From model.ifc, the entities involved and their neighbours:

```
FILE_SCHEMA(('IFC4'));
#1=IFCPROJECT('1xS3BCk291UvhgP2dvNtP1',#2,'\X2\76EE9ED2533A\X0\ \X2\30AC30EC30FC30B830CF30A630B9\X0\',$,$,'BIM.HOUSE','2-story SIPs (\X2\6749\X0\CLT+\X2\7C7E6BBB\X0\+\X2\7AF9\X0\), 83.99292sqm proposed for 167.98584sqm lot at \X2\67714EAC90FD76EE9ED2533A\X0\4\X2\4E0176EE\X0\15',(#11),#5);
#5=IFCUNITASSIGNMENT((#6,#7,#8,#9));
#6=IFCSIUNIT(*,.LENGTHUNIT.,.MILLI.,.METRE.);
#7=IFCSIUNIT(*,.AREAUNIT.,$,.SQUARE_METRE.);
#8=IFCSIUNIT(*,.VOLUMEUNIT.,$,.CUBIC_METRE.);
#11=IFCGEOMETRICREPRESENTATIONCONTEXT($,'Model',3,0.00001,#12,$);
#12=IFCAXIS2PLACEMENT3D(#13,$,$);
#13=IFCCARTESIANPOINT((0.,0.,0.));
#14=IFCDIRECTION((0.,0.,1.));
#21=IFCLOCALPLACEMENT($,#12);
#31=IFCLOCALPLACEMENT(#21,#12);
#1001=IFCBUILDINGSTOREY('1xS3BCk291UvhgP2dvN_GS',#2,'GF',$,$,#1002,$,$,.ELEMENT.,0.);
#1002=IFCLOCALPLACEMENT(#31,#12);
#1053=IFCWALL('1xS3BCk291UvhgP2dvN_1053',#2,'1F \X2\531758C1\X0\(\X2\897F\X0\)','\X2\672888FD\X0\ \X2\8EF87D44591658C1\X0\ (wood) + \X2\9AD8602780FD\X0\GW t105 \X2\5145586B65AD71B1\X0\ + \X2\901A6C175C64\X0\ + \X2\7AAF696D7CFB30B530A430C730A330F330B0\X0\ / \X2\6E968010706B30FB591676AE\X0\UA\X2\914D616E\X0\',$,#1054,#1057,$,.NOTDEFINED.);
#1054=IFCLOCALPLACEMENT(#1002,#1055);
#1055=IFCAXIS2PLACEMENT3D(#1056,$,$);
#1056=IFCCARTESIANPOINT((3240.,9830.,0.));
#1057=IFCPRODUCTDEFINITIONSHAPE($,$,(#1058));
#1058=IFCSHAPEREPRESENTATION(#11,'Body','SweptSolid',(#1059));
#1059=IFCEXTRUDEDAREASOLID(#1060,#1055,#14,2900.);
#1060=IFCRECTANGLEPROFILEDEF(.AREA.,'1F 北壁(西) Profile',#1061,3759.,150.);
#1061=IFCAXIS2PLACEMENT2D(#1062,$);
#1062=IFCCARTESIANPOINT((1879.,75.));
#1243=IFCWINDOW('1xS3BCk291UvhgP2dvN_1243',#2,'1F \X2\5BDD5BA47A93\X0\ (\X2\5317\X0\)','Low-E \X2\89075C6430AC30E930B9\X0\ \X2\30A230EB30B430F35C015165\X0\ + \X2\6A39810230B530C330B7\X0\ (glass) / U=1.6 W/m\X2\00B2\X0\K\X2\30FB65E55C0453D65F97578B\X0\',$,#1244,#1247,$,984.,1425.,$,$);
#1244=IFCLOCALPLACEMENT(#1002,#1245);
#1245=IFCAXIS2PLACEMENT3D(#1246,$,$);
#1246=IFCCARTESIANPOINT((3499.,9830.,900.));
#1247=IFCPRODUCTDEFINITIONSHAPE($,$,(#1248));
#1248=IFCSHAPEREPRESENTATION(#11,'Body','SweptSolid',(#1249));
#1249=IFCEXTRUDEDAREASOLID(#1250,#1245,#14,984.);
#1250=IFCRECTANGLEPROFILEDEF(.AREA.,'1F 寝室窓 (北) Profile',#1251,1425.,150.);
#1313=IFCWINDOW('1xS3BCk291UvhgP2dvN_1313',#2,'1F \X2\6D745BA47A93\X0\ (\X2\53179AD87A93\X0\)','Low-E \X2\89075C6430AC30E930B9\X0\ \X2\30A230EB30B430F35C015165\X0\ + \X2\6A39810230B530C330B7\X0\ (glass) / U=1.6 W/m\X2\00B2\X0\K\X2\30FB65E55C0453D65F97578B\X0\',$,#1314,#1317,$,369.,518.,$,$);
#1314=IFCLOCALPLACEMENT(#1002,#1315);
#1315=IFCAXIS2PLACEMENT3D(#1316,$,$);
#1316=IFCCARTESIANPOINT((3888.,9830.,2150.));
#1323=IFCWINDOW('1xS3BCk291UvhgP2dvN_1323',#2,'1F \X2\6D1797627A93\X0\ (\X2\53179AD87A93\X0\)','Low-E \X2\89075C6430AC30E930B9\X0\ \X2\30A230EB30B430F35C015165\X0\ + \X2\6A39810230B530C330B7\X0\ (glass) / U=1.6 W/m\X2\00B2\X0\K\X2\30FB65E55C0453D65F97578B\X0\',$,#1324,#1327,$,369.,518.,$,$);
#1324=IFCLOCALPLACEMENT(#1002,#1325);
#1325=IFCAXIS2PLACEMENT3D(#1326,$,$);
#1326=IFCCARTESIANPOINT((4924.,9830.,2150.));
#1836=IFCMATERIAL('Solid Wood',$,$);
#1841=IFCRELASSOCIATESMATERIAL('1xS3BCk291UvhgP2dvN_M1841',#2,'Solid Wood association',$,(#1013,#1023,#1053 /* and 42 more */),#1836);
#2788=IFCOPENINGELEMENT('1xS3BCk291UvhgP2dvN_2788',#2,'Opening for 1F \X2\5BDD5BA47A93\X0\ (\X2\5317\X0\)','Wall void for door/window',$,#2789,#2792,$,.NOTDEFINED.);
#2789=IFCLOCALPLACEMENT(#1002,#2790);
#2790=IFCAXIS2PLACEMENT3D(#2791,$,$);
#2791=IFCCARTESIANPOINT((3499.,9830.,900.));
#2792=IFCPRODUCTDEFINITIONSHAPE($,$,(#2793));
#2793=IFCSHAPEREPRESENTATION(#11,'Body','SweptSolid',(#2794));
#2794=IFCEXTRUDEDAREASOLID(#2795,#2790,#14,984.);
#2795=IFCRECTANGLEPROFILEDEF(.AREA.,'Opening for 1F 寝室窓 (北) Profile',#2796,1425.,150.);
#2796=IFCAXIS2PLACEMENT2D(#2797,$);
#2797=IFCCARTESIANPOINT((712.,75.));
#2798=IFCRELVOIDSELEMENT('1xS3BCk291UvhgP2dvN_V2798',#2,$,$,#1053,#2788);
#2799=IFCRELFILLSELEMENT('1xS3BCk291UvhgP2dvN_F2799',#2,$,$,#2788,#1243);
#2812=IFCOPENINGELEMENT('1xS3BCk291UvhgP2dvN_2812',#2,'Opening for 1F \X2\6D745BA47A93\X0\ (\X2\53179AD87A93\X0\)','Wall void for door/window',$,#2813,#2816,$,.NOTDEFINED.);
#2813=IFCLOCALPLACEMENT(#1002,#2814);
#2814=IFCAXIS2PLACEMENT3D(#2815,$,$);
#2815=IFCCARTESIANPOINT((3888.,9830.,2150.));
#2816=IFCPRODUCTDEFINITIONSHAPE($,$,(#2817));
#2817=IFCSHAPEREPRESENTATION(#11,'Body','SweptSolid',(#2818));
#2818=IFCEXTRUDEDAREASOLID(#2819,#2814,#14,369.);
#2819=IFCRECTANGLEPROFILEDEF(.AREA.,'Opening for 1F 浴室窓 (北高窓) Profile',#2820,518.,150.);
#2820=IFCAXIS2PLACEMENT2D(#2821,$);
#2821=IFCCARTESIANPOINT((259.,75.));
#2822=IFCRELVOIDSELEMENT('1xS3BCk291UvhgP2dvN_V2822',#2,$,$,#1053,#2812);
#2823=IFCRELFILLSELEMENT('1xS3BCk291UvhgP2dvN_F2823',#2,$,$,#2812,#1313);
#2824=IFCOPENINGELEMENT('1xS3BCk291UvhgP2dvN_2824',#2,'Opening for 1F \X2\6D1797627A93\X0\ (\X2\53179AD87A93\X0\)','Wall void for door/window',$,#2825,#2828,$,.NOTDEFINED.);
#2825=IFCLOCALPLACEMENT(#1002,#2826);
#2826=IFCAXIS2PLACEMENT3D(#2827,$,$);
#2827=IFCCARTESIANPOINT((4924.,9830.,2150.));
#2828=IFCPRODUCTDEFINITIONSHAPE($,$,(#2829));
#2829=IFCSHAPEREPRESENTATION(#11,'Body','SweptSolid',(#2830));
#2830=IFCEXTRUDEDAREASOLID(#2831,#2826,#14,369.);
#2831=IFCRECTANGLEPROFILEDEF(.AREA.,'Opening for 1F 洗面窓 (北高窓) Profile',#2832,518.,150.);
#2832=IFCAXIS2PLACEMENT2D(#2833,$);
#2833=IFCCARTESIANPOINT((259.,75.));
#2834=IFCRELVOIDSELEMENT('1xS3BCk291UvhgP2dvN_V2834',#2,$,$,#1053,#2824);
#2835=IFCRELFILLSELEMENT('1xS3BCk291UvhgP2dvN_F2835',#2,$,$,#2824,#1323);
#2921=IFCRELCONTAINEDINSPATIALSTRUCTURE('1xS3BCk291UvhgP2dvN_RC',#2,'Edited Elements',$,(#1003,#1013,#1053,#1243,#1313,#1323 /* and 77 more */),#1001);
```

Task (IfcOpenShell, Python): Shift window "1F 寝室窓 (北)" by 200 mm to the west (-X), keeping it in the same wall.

```python
import ifcopenshell
import ifcopenshell.api.geometry
import ifcopenshell.util.placement
import ifcopenshell.util.unit

model = ifcopenshell.open("model.ifc")
unit_scale = ifcopenshell.util.unit.calculate_unit_scale(model)

window = model.by_guid("1xS3BCk291UvhgP2dvN_1243")
opening = window.FillsVoids[0].RelatingOpeningElement
wall = opening.VoidsElements[0].RelatingBuildingElement

wall_matrix = ifcopenshell.util.placement.get_local_placement(wall.ObjectPlacement)
shift = wall_matrix[:3, 0] * -0.2 / unit_scale
before = ifcopenshell.util.placement.get_local_placement(window.ObjectPlacement)[:3, 3].copy()

# The window is not placed relative to its opening, so move both.
for product in (opening, window):
    matrix = ifcopenshell.util.placement.get_local_placement(product.ObjectPlacement)
    matrix[:3, 3] += shift
    ifcopenshell.api.geometry.edit_object_placement(model, product=product, matrix=matrix, is_si=False)

after = ifcopenshell.util.placement.get_local_placement(window.ObjectPlacement)[:3, 3]
print("window moved by", (after - before).round(3) + 0.0)

model.write("model_updated.ifc")
```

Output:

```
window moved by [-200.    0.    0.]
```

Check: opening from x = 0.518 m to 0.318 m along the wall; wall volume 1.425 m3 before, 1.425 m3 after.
